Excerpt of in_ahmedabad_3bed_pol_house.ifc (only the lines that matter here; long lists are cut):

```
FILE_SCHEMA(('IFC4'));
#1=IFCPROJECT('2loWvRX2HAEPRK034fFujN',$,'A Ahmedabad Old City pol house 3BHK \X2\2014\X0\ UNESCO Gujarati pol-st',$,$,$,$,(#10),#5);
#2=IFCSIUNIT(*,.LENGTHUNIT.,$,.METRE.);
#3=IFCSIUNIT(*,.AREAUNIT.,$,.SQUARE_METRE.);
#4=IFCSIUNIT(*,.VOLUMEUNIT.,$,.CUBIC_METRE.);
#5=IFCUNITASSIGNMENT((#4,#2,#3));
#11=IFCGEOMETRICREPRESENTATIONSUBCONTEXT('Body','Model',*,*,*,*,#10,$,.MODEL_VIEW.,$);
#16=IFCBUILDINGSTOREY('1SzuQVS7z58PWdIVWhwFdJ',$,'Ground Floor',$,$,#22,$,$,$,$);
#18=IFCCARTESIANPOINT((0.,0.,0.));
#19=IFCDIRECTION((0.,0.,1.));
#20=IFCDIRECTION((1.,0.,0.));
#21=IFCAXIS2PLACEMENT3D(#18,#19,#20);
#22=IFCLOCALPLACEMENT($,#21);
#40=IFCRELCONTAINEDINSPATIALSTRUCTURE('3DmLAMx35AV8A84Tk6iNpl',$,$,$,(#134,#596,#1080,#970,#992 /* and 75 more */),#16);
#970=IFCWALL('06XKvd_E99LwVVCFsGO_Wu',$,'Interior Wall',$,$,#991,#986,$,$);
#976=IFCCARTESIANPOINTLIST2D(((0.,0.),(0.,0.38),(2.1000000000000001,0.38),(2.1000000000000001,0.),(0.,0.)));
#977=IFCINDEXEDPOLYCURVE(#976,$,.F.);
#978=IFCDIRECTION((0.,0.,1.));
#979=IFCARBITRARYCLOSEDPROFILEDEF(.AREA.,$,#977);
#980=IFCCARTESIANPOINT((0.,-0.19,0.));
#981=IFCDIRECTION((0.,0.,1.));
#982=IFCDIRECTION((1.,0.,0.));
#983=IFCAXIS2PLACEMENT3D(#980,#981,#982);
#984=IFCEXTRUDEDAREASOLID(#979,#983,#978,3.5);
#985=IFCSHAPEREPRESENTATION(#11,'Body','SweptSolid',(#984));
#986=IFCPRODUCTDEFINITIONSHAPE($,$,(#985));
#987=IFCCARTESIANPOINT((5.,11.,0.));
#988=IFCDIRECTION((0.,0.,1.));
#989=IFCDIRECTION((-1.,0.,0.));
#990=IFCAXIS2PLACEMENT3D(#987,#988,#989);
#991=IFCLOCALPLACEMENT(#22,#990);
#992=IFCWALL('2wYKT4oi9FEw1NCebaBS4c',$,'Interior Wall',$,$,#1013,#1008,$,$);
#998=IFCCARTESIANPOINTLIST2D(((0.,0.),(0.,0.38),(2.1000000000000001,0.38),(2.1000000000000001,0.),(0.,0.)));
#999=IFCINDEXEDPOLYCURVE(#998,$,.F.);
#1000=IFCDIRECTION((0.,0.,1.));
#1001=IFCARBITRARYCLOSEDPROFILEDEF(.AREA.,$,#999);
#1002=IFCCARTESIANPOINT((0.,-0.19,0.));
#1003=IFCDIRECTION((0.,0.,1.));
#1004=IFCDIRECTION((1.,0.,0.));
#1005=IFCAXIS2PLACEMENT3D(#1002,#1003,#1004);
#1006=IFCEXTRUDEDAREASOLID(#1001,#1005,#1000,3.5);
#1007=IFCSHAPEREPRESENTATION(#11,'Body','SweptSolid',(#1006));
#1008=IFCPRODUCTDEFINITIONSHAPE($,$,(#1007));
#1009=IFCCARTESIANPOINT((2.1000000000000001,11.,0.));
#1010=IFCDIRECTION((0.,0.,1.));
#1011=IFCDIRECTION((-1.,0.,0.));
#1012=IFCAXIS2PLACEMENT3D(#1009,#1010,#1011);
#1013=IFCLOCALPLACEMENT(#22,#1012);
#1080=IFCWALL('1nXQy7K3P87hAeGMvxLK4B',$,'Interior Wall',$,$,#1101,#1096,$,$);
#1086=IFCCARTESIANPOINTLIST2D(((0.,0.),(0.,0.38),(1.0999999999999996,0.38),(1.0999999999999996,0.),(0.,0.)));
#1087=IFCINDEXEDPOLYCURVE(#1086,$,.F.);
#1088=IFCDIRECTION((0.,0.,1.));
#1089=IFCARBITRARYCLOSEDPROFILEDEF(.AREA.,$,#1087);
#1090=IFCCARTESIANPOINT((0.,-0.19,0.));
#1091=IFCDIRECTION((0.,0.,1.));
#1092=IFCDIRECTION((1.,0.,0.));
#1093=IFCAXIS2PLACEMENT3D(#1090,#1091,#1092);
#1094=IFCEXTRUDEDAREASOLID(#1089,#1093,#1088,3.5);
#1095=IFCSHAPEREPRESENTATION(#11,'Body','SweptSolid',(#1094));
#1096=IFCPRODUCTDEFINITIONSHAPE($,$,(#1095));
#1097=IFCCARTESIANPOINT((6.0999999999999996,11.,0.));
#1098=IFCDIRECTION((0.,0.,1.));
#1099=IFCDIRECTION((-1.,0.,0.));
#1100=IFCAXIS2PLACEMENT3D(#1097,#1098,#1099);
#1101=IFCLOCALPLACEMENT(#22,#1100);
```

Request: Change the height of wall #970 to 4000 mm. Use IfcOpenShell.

```python
import ifcopenshell
import ifcopenshell.geom
import ifcopenshell.util.representation
import ifcopenshell.util.shape
import ifcopenshell.util.unit

model = ifcopenshell.open("in_ahmedabad_3bed_pol_house.ifc")
unit_scale = ifcopenshell.util.unit.calculate_unit_scale(model)
settings = ifcopenshell.geom.settings()


def volume(element):
    """Net volume in cubic metres, openings subtracted."""
    shape = ifcopenshell.geom.create_shape(settings, element)
    return ifcopenshell.util.shape.get_volume(shape.geometry)


wall = model.by_id(970)
before = volume(wall)

body = ifcopenshell.util.representation.get_representation(wall, "Model", "Body")
solid = body.Items[0]
old_height = solid.Depth
solid.Depth = 4 / unit_scale
after = volume(wall)

print(f"height {old_height:g} -> {solid.Depth:g}, volume {before:.3f} -> {after:.3f} m3")

model.write("in_ahmedabad_3bed_pol_house-out.ifc")
```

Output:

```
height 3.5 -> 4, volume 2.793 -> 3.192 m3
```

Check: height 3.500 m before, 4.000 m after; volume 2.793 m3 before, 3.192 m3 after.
